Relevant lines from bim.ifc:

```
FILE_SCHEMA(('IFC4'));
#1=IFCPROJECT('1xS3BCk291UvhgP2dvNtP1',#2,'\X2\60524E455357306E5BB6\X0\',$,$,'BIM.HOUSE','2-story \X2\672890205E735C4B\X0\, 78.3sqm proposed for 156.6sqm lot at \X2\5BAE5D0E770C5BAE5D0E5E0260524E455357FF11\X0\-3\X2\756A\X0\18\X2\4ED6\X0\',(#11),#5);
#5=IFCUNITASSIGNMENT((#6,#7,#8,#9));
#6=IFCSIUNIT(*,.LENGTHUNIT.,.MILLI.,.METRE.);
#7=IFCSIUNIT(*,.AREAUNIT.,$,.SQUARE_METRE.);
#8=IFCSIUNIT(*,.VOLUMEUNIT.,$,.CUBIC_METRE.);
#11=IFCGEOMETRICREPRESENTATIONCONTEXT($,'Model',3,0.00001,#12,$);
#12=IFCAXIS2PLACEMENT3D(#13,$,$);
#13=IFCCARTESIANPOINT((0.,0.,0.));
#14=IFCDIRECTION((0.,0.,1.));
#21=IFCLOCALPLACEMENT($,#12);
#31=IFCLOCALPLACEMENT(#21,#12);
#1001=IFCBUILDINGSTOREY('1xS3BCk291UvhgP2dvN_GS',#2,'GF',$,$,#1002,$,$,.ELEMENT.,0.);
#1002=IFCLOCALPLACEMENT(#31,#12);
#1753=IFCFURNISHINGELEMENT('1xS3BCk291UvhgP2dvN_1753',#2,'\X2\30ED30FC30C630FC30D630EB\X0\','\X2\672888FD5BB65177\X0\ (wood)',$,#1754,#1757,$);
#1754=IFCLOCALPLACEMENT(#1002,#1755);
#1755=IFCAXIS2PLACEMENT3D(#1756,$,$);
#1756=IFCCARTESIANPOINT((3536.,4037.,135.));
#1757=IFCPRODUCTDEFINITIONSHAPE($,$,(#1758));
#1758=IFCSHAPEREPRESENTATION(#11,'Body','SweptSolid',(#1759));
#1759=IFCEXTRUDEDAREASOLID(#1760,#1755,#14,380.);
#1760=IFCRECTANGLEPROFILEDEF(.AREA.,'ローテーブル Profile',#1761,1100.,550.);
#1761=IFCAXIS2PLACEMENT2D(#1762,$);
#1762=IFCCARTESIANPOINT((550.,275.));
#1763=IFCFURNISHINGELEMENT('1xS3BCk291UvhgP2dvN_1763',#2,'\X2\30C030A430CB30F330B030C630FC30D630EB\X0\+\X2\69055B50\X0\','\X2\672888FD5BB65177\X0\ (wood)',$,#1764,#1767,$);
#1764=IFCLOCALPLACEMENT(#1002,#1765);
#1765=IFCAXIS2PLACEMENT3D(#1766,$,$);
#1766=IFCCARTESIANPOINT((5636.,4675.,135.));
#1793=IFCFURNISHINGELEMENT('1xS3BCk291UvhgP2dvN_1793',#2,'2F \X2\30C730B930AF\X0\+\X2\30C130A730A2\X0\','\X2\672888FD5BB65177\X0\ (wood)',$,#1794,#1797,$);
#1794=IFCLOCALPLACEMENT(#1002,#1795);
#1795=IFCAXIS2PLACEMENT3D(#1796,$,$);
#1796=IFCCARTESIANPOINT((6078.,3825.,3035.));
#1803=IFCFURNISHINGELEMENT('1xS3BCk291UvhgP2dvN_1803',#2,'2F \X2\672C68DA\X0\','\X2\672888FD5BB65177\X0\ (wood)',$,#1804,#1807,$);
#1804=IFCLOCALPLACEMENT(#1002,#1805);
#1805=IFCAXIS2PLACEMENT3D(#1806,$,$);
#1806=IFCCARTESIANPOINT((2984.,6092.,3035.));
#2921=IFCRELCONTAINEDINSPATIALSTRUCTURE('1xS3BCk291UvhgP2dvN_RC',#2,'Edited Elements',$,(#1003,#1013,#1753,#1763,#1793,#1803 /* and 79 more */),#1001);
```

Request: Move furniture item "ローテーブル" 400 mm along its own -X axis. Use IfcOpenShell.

```python
import ifcopenshell
import ifcopenshell.api.geometry
import ifcopenshell.util.placement
import ifcopenshell.util.unit

model = ifcopenshell.open("bim.ifc")
unit_scale = ifcopenshell.util.unit.calculate_unit_scale(model)

item = model.by_guid("1xS3BCk291UvhgP2dvN_1753")
matrix = ifcopenshell.util.placement.get_local_placement(item.ObjectPlacement)
matrix[:3, 3] -= matrix[:3, 0] * 0.4 / unit_scale
ifcopenshell.api.geometry.edit_object_placement(model, product=item, matrix=matrix, is_si=False)

print(ifcopenshell.util.placement.get_local_placement(item.ObjectPlacement).round(3) + 0.0)

model.write("bim-out.ifc")
```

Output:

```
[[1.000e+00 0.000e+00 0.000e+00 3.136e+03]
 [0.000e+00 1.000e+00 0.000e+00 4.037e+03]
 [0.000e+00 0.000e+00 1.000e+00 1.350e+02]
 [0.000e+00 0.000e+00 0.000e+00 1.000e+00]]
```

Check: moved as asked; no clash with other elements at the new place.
